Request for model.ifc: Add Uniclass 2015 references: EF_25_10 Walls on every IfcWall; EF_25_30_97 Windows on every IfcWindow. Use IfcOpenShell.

First a look at what the model holds.

```python
import ifcopenshell

model = ifcopenshell.open("model.ifc")
print(model.schema)
print("classifications:", [c.Name for c in model.by_type("IfcClassification")])
for ifc_class in ("IfcDoor", "IfcRoof", "IfcStair", "IfcWall", "IfcWindow"):
    print(ifc_class, len(model.by_type(ifc_class)))
```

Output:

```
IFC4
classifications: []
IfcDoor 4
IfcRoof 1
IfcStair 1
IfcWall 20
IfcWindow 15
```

```python
import ifcopenshell
import ifcopenshell.api.classification

model = ifcopenshell.open("model.ifc")

system = ifcopenshell.api.classification.add_classification(model, classification="Uniclass 2015")

codes = {
    "IfcWall": ("EF_25_10", "Walls"),
    "IfcWindow": ("EF_25_30_97", "Windows"),
}
for ifc_class, (code, name) in codes.items():
    products = model.by_type(ifc_class)
    ifcopenshell.api.classification.add_reference(
        model, products=products, classification=system, identification=code, name=name
    )
    print(code, len(products))

model.write("model_v2.ifc")
```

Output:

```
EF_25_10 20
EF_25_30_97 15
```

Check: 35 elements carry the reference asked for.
